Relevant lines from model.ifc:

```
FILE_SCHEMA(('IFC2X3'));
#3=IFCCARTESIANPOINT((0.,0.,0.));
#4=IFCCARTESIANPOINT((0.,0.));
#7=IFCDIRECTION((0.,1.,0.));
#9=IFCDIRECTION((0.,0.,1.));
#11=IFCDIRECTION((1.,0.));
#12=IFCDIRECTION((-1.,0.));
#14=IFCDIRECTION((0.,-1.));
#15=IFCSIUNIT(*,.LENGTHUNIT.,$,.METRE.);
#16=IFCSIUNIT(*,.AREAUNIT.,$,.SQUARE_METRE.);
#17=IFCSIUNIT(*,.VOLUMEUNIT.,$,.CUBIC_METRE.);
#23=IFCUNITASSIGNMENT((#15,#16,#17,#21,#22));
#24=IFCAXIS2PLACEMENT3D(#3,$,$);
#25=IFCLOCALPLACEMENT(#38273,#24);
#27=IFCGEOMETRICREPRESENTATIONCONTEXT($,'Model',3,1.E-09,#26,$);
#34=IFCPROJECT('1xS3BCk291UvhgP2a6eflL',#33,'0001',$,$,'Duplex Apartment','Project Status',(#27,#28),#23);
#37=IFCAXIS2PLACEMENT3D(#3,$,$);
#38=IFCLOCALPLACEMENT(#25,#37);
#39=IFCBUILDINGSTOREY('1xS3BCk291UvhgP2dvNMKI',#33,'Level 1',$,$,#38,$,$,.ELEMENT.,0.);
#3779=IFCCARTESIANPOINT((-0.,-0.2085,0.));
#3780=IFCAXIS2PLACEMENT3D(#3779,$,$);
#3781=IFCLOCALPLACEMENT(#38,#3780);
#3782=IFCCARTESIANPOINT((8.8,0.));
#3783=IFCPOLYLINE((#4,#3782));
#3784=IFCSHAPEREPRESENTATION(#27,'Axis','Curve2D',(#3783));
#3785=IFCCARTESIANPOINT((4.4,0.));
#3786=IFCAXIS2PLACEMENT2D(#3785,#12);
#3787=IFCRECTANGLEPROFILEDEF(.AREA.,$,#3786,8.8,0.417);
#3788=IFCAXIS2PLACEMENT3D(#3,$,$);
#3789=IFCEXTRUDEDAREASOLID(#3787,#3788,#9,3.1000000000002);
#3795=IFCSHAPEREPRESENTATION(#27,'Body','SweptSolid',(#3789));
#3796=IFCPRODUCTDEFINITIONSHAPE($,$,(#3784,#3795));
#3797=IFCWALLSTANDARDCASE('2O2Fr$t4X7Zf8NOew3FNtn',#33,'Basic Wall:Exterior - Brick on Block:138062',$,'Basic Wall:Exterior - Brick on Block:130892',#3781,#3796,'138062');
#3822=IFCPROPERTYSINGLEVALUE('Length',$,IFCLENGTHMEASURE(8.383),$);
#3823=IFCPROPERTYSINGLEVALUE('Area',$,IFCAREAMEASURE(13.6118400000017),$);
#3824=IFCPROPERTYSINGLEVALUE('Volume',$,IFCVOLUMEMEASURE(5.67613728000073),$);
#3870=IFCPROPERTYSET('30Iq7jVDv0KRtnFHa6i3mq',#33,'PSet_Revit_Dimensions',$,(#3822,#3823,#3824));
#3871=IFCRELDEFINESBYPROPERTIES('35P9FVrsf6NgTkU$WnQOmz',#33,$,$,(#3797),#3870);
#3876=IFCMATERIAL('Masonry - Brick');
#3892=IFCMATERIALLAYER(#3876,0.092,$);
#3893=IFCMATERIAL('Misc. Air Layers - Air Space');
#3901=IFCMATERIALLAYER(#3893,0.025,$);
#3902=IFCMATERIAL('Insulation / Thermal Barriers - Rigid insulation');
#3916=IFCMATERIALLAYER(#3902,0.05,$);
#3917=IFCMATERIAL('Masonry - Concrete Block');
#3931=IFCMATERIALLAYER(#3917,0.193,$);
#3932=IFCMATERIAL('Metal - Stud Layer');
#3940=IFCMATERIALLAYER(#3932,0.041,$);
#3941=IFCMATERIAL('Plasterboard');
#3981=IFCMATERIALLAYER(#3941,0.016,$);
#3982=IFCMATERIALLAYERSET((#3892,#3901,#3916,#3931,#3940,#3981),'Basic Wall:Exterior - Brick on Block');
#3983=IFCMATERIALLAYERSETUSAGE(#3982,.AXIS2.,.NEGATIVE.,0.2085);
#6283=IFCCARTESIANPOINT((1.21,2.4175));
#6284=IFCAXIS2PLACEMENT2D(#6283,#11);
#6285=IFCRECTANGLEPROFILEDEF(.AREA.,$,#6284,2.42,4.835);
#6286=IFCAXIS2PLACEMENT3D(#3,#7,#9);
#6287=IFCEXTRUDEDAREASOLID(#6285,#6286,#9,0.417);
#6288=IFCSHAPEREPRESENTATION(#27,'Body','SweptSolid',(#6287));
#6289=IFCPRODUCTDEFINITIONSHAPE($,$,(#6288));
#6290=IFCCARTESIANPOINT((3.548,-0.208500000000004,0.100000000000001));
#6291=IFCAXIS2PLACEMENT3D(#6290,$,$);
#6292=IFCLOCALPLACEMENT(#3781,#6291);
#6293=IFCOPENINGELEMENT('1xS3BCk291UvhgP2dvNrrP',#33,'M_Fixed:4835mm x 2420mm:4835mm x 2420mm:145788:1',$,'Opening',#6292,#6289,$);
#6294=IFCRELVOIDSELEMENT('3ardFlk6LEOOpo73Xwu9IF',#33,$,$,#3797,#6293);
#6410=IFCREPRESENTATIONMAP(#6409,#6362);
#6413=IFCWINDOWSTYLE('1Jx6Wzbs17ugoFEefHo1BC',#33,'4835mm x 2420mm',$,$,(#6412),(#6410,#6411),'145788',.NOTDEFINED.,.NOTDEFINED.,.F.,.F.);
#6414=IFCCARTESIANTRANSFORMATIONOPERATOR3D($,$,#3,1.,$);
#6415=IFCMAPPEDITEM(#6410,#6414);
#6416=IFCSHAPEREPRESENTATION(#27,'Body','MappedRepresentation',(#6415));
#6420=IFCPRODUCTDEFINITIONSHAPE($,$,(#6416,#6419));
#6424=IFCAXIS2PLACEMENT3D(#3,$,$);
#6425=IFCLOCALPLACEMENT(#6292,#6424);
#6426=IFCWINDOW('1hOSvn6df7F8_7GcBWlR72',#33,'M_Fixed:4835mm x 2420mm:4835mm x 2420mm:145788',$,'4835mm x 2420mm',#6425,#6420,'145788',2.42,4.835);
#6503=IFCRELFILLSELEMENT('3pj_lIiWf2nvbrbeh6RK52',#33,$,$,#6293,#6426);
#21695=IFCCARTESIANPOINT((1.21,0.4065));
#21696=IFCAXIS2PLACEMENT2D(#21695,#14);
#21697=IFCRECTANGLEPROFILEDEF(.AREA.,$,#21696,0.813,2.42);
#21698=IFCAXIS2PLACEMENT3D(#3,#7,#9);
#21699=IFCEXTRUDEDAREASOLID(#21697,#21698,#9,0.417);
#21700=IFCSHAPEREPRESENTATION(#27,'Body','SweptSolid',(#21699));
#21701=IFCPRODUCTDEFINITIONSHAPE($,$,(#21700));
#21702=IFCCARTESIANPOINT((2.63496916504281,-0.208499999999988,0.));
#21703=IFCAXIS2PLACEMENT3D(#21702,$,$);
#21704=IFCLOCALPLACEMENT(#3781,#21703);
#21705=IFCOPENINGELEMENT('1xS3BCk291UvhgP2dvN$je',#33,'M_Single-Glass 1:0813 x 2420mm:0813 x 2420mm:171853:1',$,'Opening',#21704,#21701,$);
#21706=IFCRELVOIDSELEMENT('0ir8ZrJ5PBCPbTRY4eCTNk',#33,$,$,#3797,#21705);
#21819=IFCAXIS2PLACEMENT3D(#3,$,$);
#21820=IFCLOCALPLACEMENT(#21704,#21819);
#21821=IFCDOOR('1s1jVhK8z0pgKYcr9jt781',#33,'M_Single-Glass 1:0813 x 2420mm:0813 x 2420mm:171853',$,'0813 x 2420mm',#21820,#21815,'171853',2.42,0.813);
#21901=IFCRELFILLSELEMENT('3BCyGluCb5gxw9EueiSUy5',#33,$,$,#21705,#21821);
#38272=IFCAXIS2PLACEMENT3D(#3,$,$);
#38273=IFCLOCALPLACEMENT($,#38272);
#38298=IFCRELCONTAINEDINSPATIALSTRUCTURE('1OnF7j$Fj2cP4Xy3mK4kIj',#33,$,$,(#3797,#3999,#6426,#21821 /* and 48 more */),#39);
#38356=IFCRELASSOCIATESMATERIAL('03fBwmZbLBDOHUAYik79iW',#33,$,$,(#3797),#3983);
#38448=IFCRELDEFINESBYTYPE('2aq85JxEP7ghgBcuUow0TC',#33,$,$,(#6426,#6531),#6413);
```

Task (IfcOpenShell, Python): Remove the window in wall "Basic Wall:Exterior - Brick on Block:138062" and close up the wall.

```python
import ifcopenshell
import ifcopenshell.api.feature
import ifcopenshell.api.pset
import ifcopenshell.api.root
import ifcopenshell.geom
import ifcopenshell.util.element
import ifcopenshell.util.shape
import ifcopenshell.util.unit

model = ifcopenshell.open("model.ifc")
area_scale = ifcopenshell.util.unit.calculate_unit_scale(model, "AREAUNIT")
volume_scale = ifcopenshell.util.unit.calculate_unit_scale(model, "VOLUMEUNIT")
settings = ifcopenshell.geom.settings()


def volume(element):
    """Net volume in cubic metres, openings subtracted."""
    shape = ifcopenshell.geom.create_shape(settings, element)
    return ifcopenshell.util.shape.get_volume(shape.geometry)


window = model.by_guid("1hOSvn6df7F8_7GcBWlR72")
opening = window.FillsVoids[0].RelatingOpeningElement
wall = opening.VoidsElements[0].RelatingBuildingElement
before = volume(wall)

ifcopenshell.api.root.remove_product(model, product=window)
ifcopenshell.api.feature.remove_feature(model, feature=opening)

after = volume(wall)
thickness = 0.417  # wall thickness in metres

# Update the wall's stored quantities.
pset = model.by_id(ifcopenshell.util.element.get_pset(wall, "PSet_Revit_Dimensions", should_inherit=False)["id"])
ifcopenshell.api.pset.edit_pset(model, pset=pset, properties={
    "Area": model.create_entity("IfcAreaMeasure", after / thickness / area_scale),
    "Volume": model.create_entity("IfcVolumeMeasure", after / volume_scale),
})

print(f"wall volume {before:.3f} -> {after:.3f} m3")

model.write("model_rev.ifc")
```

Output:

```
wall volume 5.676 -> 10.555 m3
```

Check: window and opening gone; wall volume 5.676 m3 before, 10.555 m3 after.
